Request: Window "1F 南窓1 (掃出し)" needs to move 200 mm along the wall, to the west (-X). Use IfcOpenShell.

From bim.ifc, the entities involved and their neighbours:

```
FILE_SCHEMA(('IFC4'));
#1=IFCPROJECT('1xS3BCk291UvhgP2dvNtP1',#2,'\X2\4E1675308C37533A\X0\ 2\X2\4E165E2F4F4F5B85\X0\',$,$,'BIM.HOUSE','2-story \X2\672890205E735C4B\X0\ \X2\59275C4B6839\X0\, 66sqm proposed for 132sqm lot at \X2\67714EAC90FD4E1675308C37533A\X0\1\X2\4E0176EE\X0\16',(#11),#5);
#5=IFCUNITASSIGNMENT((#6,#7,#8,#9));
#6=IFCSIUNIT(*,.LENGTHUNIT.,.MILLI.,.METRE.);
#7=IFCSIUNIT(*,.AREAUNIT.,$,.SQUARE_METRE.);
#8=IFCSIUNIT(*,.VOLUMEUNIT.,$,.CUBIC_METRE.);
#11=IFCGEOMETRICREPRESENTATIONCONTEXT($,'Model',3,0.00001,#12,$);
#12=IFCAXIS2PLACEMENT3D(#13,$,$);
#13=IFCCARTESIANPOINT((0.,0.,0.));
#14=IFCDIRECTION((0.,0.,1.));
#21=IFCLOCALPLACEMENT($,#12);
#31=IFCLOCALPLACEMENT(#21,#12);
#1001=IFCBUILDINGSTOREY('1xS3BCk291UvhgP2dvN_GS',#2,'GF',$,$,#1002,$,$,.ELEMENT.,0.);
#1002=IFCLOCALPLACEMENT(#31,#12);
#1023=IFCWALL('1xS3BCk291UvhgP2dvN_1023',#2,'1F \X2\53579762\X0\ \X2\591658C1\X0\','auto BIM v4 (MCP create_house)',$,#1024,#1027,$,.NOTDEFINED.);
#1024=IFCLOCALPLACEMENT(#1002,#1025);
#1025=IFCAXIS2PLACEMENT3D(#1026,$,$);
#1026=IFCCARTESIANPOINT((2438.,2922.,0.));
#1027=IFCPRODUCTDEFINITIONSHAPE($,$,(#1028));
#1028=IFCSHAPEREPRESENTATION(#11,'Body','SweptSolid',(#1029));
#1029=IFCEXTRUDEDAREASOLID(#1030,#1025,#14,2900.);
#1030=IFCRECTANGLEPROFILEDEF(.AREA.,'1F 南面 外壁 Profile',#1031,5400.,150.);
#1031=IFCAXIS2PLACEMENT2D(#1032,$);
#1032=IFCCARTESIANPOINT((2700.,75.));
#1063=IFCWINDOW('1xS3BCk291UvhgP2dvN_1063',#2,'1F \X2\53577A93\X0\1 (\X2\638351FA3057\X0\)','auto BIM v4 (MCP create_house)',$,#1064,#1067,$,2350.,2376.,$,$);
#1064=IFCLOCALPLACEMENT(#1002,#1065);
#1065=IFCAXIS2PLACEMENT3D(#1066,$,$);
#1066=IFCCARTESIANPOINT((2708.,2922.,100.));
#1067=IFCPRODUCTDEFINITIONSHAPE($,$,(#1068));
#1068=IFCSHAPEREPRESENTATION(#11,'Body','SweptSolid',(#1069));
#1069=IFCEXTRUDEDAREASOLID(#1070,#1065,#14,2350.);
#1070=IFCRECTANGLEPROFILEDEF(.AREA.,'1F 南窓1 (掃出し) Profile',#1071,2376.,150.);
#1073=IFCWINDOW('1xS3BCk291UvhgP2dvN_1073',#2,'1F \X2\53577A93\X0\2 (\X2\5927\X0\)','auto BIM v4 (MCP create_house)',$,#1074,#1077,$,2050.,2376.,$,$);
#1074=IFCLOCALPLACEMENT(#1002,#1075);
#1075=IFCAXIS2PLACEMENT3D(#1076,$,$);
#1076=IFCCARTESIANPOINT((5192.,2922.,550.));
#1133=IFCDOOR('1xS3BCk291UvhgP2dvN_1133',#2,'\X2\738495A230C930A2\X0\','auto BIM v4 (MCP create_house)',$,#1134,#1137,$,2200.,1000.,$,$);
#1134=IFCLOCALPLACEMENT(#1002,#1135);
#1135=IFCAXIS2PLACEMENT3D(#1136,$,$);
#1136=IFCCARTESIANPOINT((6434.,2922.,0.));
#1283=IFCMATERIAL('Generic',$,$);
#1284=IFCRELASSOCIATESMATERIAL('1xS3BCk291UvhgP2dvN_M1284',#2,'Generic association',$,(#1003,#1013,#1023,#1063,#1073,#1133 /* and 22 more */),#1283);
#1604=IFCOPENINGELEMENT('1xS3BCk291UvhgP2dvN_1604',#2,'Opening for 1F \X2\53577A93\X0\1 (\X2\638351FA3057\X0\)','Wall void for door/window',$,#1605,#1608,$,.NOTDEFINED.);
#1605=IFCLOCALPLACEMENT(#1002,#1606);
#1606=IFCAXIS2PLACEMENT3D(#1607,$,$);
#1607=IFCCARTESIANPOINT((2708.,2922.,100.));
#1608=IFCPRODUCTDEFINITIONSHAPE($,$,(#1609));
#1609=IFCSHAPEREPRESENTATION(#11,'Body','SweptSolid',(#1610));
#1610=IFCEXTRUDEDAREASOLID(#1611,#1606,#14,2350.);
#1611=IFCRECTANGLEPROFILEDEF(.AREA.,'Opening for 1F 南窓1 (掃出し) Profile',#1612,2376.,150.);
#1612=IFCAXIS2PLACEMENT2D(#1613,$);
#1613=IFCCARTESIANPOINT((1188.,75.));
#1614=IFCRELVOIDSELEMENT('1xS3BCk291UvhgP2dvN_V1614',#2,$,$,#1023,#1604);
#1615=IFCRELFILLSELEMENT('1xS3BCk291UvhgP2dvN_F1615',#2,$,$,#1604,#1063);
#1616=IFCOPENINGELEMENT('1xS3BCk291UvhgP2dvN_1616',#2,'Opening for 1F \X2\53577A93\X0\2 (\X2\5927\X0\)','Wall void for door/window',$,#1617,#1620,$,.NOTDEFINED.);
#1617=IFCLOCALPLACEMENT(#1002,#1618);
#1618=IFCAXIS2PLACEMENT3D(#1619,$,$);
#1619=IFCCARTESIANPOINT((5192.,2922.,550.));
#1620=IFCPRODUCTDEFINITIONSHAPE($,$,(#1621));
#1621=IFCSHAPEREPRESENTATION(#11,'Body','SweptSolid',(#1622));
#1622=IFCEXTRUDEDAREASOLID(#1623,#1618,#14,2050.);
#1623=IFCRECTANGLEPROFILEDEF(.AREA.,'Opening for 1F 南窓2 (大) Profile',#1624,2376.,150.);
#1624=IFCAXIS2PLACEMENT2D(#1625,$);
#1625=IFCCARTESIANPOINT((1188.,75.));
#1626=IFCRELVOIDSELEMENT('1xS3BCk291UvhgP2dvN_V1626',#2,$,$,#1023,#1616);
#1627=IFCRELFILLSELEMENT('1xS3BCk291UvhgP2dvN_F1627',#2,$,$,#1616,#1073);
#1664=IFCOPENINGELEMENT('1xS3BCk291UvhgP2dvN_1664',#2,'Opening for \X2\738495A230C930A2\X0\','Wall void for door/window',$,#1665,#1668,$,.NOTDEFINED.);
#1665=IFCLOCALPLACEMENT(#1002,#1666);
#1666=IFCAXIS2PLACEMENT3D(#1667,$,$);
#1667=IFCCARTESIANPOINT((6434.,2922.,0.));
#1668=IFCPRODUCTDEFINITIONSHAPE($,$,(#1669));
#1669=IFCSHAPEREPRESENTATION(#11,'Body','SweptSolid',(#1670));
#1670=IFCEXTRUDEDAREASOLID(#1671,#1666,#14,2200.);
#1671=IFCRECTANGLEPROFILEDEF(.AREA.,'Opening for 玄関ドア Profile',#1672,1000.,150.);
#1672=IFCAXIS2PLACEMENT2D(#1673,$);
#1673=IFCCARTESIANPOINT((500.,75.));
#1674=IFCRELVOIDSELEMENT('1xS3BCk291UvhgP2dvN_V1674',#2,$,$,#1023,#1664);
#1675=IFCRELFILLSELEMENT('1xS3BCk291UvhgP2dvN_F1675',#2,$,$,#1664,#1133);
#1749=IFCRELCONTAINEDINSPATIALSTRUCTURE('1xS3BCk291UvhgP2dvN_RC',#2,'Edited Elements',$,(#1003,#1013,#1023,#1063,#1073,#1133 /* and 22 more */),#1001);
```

```python
import ifcopenshell
import ifcopenshell.api.geometry
import ifcopenshell.util.placement
import ifcopenshell.util.unit

model = ifcopenshell.open("bim.ifc")
unit_scale = ifcopenshell.util.unit.calculate_unit_scale(model)

window = model.by_guid("1xS3BCk291UvhgP2dvN_1063")
opening = window.FillsVoids[0].RelatingOpeningElement
wall = opening.VoidsElements[0].RelatingBuildingElement

wall_matrix = ifcopenshell.util.placement.get_local_placement(wall.ObjectPlacement)
shift = wall_matrix[:3, 0] * -0.2 / unit_scale
before = ifcopenshell.util.placement.get_local_placement(window.ObjectPlacement)[:3, 3].copy()

# The window is not placed relative to its opening, so move both.
for product in (opening, window):
    matrix = ifcopenshell.util.placement.get_local_placement(product.ObjectPlacement)
    matrix[:3, 3] += shift
    ifcopenshell.api.geometry.edit_object_placement(model, product=product, matrix=matrix, is_si=False)

after = ifcopenshell.util.placement.get_local_placement(window.ObjectPlacement)[:3, 3]
print("window moved by", (after - before).round(3) + 0.0)

model.write("bim_v2.ifc")
```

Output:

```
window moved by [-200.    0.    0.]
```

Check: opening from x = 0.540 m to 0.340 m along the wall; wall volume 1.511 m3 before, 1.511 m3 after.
